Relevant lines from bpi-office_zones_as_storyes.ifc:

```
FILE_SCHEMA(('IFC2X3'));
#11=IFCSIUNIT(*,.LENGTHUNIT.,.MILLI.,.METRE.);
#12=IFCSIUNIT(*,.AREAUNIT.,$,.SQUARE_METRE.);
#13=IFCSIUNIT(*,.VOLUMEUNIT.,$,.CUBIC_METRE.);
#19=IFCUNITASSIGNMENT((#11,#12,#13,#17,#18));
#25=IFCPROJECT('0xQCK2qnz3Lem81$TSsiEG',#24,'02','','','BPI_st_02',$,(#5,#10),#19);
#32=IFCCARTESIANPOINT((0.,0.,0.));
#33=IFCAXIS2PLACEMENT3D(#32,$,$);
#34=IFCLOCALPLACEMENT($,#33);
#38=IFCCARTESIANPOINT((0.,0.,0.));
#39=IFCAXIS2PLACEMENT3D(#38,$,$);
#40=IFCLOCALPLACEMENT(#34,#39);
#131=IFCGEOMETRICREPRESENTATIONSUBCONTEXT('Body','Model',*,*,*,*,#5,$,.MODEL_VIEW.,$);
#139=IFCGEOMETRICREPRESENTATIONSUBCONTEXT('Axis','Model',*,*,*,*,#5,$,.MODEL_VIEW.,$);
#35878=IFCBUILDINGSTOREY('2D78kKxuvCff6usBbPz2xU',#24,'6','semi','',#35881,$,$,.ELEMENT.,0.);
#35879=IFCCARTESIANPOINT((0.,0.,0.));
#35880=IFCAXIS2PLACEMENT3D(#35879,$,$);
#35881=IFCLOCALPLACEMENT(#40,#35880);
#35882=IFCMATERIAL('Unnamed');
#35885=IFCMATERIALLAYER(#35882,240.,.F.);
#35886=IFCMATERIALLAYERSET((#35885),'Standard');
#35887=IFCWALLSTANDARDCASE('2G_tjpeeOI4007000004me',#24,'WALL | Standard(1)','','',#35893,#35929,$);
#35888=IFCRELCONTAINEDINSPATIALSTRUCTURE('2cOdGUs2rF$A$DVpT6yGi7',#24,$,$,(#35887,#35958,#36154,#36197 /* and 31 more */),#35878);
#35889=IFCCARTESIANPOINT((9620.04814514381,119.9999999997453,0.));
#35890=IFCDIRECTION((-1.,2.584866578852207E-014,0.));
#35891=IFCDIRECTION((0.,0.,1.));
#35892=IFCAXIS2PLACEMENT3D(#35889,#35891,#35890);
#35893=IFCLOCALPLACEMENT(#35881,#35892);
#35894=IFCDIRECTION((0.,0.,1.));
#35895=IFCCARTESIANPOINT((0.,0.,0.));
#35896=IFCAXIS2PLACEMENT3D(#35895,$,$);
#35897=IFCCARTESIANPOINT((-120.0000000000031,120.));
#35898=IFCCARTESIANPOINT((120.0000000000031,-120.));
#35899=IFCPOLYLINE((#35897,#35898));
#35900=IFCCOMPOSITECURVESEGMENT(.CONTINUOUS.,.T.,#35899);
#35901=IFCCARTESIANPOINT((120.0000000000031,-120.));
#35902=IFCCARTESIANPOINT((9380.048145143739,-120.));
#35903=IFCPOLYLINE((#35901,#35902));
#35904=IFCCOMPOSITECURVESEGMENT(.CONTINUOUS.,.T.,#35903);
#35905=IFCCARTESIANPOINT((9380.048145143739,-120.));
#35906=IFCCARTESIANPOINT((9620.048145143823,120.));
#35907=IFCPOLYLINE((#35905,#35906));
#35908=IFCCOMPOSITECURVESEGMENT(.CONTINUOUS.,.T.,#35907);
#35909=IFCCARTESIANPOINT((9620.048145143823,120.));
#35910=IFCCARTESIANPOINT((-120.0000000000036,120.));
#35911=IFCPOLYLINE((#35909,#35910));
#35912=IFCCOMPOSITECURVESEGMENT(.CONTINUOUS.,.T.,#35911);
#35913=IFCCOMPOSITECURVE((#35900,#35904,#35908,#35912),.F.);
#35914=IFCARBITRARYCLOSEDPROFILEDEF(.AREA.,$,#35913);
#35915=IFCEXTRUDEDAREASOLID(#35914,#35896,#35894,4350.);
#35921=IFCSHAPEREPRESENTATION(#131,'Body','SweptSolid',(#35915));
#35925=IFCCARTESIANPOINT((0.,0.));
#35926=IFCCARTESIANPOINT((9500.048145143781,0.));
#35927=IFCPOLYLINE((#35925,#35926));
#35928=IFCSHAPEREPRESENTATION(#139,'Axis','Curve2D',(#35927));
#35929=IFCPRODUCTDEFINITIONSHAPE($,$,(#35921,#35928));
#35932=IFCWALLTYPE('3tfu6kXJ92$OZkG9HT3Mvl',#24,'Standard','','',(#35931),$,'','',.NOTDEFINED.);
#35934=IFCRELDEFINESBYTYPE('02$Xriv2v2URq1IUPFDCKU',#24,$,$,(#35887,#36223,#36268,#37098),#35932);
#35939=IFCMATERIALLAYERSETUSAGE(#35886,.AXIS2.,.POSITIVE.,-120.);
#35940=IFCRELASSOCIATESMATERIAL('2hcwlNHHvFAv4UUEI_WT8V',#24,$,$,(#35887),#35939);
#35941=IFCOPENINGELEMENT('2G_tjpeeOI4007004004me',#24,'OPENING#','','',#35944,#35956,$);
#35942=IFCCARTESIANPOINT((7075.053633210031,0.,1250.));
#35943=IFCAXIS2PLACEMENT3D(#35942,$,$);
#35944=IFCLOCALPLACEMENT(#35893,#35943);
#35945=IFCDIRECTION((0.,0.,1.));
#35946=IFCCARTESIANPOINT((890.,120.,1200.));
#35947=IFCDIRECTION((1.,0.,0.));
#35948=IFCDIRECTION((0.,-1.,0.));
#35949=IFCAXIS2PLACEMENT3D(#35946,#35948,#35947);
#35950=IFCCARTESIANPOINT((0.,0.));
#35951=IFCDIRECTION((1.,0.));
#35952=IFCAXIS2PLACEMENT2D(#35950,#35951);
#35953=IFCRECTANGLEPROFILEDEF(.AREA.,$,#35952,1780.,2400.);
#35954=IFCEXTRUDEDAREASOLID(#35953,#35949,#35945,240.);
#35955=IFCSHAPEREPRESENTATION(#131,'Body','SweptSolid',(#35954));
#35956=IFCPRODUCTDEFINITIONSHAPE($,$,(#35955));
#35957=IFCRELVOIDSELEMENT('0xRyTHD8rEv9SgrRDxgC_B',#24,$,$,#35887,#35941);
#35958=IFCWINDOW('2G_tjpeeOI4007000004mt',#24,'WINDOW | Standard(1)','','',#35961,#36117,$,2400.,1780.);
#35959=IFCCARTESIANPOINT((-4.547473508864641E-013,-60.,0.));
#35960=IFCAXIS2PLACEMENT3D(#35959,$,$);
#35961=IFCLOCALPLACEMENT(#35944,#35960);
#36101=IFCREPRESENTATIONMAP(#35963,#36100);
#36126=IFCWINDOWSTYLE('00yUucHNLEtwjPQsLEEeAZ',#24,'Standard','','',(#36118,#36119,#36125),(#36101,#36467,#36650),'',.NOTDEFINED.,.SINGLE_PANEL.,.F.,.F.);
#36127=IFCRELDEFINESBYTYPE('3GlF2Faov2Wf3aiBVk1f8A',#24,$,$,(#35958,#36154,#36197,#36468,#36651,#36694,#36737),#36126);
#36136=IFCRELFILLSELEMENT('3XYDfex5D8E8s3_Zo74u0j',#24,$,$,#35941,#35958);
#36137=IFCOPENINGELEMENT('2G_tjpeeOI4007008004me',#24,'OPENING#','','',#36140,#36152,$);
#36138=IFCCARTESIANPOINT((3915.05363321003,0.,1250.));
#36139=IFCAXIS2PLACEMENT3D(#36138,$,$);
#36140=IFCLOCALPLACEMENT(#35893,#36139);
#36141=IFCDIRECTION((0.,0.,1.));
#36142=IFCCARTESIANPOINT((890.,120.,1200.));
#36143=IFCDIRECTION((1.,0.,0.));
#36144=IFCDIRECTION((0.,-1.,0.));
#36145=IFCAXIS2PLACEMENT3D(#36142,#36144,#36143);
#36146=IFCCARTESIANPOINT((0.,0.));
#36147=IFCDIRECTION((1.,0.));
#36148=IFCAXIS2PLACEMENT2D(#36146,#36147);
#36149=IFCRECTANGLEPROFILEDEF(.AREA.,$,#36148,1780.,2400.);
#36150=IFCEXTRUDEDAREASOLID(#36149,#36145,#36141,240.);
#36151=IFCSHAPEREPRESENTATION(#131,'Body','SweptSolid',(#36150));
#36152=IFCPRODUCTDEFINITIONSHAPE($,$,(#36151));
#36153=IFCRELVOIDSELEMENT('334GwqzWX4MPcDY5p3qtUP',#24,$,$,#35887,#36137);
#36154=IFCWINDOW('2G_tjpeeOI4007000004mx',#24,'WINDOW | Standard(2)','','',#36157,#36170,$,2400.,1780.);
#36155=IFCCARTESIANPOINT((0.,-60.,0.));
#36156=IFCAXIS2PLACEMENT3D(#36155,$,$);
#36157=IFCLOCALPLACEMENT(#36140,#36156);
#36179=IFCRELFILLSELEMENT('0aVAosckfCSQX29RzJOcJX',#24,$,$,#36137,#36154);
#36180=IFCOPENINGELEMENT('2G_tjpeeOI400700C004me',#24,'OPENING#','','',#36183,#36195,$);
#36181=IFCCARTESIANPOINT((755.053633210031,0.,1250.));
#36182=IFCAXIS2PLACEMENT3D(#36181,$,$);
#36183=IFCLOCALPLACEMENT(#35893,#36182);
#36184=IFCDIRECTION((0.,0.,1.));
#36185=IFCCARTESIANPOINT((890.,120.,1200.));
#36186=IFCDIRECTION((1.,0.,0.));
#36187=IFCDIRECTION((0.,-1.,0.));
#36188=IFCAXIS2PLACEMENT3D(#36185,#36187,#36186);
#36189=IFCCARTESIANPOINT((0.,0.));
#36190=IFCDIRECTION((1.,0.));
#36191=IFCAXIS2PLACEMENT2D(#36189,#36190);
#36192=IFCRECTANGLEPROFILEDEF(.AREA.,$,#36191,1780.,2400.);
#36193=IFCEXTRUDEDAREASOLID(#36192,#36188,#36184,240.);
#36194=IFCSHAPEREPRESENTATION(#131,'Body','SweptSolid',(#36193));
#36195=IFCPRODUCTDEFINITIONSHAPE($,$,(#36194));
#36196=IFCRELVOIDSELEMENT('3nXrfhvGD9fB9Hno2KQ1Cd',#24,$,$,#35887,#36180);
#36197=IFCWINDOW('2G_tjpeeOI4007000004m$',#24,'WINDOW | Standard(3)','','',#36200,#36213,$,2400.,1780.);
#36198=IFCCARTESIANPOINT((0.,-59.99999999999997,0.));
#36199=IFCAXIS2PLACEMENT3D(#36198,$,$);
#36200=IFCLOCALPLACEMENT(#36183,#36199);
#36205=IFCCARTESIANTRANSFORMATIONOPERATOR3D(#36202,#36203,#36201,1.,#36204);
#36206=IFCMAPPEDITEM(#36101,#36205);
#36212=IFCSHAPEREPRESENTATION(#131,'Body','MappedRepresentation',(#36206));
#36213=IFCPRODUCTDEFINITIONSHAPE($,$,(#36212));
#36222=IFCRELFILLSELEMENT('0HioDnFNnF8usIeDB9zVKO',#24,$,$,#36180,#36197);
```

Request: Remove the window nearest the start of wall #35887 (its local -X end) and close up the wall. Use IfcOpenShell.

```python
import ifcopenshell
import ifcopenshell.api.feature
import ifcopenshell.api.root
import ifcopenshell.geom
import ifcopenshell.util.shape

model = ifcopenshell.open("bpi-office_zones_as_storyes.ifc")
settings = ifcopenshell.geom.settings()


def volume(element):
    """Net volume in cubic metres, openings subtracted."""
    shape = ifcopenshell.geom.create_shape(settings, element)
    return ifcopenshell.util.shape.get_volume(shape.geometry)


window = model.by_id(36197)
opening = window.FillsVoids[0].RelatingOpeningElement
wall = opening.VoidsElements[0].RelatingBuildingElement
before = volume(wall)

ifcopenshell.api.root.remove_product(model, product=window)
ifcopenshell.api.feature.remove_feature(model, feature=opening)

after = volume(wall)

print(f"wall volume {before:.3f} -> {after:.3f} m3")

model.write("bpi-office_zones_as_storyes_v2.ifc")
```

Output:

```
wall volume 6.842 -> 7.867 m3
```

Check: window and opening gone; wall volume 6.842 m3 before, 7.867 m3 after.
